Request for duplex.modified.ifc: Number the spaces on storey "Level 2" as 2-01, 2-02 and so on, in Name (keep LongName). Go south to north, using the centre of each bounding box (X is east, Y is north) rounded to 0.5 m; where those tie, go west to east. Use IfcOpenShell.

First a look at what the model holds.

```python
import ifcopenshell
import ifcopenshell.util.element
import ifcopenshell.util.placement

model = ifcopenshell.open("duplex.modified.ifc")
print(model.schema)
storey = next(s for s in model.by_type("IfcBuildingStorey") if s.Name == "Level 2")
spaces = [e for e in ifcopenshell.util.element.get_decomposition(storey) if e.is_a("IfcSpace")]
for e in sorted(spaces, key=lambda e: e.id()):
    origin = ifcopenshell.util.placement.get_local_placement(e.ObjectPlacement)[:3, 3]
    print(e.id(), e.Name, e.LongName, origin.round(2) + 0.0, sep=" | ")
```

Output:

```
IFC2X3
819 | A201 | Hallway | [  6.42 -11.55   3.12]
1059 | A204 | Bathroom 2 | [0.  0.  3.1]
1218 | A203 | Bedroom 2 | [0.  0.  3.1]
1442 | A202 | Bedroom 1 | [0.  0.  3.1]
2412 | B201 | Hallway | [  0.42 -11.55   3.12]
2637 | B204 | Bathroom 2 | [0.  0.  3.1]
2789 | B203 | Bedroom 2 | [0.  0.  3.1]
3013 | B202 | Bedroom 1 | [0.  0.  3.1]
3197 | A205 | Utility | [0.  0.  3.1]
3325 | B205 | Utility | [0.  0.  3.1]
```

```python
import ifcopenshell
import ifcopenshell.geom
import ifcopenshell.util.element
import ifcopenshell.util.shape

model = ifcopenshell.open("duplex.modified.ifc")
settings = ifcopenshell.geom.settings()
settings.set("use-world-coords", True)


def centre(element):
    shape = ifcopenshell.geom.create_shape(settings, element)
    return ifcopenshell.util.shape.get_bbox_centroid(shape.geometry)


storey = next(s for s in model.by_type("IfcBuildingStorey") if s.Name == "Level 2")
spaces = [e for e in ifcopenshell.util.element.get_decomposition(storey) if e.is_a("IfcSpace")]

# Insertion points can sit at a corner or the storey origin, so sort by the geometry (in metres).
centres = {e: centre(e) for e in spaces}
spaces.sort(key=lambda e: (round(centres[e][1] / 0.5), centres[e][0]))

for i, e in enumerate(spaces, start=1):
    number = f"2-{i:02d}"
    e.Name = number
    print(e.id(), number)

model.write("duplex.modified_edited.ifc")
```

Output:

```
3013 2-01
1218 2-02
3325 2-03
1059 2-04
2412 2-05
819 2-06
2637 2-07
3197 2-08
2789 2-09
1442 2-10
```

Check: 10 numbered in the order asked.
